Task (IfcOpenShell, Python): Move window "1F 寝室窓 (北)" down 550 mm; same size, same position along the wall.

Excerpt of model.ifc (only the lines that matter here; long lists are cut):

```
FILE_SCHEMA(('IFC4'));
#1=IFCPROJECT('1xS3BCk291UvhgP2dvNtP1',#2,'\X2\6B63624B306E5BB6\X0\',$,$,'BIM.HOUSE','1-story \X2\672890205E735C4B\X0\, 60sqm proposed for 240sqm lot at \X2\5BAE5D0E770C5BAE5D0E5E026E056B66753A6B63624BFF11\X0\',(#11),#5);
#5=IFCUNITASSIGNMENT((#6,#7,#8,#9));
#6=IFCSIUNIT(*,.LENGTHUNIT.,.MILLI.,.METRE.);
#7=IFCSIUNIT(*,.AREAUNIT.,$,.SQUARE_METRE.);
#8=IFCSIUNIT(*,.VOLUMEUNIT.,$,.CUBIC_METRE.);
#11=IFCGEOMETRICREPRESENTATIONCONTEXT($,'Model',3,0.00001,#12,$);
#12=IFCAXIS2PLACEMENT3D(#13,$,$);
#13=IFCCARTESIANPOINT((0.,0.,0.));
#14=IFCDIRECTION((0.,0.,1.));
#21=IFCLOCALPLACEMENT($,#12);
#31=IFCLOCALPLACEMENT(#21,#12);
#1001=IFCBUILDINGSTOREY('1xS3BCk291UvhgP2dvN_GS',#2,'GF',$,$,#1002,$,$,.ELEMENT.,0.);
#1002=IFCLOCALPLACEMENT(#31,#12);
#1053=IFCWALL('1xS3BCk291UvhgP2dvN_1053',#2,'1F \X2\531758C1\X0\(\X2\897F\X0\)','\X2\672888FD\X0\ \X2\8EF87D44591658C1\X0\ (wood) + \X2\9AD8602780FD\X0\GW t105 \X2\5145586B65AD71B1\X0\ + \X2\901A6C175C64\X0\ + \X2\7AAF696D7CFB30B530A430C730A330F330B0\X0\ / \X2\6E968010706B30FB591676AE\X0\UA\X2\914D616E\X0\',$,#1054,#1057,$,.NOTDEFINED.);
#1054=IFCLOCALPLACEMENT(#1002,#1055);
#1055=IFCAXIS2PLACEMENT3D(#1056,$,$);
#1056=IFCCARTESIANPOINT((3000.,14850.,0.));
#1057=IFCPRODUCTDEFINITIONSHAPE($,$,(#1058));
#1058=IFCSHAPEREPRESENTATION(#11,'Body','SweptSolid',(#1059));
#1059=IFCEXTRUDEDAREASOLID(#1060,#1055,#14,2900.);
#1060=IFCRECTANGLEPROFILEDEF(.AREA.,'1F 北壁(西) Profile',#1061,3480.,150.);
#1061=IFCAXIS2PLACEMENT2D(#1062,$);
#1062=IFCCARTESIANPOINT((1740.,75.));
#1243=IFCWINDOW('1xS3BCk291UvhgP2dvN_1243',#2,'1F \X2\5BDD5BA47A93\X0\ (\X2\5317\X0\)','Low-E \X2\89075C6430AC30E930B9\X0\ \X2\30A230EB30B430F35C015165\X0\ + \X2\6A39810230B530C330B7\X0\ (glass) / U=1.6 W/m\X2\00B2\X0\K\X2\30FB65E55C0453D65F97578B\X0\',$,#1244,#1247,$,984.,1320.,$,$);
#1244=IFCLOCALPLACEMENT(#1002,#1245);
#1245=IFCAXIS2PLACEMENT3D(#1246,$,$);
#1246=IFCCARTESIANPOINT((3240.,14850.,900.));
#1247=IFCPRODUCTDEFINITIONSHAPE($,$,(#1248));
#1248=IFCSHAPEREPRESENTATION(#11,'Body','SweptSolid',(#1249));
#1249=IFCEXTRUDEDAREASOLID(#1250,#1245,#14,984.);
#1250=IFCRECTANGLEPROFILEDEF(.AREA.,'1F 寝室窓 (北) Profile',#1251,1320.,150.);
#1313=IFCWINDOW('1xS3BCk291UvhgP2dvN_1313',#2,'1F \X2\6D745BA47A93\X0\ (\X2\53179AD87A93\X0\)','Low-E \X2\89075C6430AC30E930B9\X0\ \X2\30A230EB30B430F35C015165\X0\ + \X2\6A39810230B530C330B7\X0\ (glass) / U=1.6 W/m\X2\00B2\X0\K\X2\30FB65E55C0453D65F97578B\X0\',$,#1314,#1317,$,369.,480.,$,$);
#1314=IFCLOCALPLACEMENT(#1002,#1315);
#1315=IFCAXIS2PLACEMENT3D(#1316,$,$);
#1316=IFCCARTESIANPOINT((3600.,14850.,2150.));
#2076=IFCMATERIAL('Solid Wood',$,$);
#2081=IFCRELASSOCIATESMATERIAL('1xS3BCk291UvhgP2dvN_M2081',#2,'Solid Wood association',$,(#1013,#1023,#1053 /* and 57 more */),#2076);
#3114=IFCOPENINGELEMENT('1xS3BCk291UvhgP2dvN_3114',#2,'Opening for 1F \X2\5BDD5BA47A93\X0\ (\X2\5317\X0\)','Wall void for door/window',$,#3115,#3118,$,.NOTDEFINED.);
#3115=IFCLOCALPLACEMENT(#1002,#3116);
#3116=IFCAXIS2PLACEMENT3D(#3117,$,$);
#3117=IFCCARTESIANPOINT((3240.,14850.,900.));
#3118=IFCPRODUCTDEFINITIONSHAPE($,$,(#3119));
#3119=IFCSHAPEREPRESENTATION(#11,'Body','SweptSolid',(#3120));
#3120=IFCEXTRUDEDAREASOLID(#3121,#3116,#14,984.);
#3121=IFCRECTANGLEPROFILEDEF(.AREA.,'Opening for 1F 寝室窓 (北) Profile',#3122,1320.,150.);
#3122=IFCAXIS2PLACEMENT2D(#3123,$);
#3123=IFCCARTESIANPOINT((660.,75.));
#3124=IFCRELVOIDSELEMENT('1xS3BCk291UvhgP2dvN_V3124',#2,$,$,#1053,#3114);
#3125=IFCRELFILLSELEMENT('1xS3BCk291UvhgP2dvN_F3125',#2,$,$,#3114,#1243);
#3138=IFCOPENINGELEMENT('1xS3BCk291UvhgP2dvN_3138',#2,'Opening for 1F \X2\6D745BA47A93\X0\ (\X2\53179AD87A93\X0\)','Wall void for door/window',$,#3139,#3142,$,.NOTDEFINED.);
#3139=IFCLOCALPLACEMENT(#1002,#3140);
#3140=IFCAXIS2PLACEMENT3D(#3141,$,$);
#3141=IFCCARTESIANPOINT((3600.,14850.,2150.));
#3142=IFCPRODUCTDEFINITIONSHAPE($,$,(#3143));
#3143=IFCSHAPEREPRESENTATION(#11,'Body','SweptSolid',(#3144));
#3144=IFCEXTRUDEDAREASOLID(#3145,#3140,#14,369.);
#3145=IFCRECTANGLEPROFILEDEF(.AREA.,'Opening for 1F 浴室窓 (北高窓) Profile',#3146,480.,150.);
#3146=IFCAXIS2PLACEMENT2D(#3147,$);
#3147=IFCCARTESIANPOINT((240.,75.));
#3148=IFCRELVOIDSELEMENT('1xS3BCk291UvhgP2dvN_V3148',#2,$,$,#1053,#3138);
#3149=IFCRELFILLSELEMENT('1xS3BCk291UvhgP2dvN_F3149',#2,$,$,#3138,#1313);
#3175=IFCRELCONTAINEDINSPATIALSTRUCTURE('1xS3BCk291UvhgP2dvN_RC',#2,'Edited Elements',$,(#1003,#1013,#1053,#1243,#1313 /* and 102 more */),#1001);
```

```python
import numpy as np
import ifcopenshell
import ifcopenshell.api.geometry
import ifcopenshell.util.placement
import ifcopenshell.util.unit

model = ifcopenshell.open("model.ifc")
unit_scale = ifcopenshell.util.unit.calculate_unit_scale(model)

window = model.by_guid("1xS3BCk291UvhgP2dvN_1243")
opening = window.FillsVoids[0].RelatingOpeningElement
dz = -550.0

shift = np.array([0.0, 0.0, dz])
# The window is not placed relative to its opening, so move both.
for product in (opening, window):
    matrix = ifcopenshell.util.placement.get_local_placement(product.ObjectPlacement)
    matrix[:3, 3] += shift
    ifcopenshell.api.geometry.edit_object_placement(model, product=product, matrix=matrix, is_si=False)

print(f"moved by {dz * unit_scale:+.3f} m")

model.write("model_edited.ifc")
```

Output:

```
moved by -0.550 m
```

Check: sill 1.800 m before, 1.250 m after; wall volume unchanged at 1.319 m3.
